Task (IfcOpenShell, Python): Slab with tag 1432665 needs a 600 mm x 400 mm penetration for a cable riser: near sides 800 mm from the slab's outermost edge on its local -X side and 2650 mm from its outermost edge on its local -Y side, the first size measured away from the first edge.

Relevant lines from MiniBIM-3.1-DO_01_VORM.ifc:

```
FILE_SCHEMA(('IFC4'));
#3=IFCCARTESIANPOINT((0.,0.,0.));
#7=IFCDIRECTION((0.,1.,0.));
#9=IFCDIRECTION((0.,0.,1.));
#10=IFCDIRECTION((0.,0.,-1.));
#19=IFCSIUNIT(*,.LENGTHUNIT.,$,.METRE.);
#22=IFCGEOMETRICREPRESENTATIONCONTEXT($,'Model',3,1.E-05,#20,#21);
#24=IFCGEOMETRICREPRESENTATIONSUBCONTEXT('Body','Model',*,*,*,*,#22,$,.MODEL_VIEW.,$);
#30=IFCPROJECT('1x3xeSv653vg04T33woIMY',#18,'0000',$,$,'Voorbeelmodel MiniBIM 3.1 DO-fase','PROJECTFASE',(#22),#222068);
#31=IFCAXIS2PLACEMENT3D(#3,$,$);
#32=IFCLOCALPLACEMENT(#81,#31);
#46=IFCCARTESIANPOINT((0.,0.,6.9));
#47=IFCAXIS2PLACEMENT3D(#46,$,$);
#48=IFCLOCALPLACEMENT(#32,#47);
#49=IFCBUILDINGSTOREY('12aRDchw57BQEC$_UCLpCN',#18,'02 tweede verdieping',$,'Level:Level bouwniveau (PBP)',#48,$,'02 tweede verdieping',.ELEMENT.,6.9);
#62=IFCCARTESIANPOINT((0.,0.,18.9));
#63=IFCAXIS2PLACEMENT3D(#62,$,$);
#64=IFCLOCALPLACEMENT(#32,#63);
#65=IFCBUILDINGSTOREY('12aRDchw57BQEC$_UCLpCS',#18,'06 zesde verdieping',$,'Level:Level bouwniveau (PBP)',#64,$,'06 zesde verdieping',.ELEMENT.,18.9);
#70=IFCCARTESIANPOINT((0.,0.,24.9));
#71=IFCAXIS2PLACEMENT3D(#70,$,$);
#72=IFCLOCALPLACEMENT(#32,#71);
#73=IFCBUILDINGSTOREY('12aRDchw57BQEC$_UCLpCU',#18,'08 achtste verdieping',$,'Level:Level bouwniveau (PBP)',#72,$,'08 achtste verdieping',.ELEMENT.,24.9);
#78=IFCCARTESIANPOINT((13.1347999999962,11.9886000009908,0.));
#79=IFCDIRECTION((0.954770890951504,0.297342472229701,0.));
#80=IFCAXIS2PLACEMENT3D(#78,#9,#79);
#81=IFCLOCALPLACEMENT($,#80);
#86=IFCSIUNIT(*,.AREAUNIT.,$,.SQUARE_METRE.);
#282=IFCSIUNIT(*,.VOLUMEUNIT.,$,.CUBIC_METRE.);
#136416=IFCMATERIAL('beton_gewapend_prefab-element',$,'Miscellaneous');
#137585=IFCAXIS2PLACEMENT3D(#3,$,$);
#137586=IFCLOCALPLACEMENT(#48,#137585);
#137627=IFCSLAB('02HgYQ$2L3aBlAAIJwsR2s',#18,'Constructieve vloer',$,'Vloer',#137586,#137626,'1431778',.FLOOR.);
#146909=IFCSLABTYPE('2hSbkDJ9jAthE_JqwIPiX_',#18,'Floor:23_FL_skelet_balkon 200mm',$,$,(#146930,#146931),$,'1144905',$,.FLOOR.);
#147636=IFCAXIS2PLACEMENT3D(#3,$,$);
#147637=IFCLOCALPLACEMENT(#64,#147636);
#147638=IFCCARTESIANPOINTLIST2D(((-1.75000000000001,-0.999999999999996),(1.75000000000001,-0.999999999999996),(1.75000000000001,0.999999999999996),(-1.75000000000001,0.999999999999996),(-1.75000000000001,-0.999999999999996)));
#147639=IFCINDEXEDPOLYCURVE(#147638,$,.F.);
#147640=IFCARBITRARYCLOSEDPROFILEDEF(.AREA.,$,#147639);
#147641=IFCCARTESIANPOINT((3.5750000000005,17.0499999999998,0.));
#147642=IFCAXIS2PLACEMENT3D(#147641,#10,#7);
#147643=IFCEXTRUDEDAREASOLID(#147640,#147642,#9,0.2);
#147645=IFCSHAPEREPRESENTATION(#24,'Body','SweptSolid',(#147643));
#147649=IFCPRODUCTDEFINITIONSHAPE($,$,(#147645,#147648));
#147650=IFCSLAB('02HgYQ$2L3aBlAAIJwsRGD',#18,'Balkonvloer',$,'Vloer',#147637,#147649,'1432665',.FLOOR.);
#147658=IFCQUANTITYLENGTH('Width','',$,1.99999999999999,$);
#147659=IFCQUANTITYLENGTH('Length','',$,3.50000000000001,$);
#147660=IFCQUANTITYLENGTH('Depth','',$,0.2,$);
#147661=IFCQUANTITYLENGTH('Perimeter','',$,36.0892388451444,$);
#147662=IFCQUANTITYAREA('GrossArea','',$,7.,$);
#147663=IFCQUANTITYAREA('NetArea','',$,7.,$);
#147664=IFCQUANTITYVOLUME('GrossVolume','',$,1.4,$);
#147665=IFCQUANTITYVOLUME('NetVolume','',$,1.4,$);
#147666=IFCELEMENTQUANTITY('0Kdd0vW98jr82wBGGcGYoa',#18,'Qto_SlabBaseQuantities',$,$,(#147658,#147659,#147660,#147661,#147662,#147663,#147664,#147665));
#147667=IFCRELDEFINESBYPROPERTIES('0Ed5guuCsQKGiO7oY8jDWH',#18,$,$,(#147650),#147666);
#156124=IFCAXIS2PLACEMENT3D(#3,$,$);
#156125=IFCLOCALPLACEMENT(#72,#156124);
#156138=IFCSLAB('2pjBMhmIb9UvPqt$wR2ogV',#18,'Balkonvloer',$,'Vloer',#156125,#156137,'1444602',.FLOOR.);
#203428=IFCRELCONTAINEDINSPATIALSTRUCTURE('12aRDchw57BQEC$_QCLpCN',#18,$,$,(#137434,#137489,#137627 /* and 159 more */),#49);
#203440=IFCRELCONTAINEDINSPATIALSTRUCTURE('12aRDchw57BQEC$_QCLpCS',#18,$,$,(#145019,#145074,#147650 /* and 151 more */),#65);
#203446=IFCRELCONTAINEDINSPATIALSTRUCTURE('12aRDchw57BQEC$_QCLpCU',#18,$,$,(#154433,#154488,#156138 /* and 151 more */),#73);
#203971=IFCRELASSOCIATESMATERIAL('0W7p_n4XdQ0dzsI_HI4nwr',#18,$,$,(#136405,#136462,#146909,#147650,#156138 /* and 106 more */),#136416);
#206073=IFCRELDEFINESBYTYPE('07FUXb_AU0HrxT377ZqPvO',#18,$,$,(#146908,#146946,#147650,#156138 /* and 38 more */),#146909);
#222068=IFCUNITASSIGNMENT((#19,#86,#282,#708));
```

```python
import numpy as np
import ifcopenshell
import ifcopenshell.api.feature
import ifcopenshell.api.geometry
import ifcopenshell.api.pset
import ifcopenshell.api.root
import ifcopenshell.geom
import ifcopenshell.util.element
import ifcopenshell.util.placement
import ifcopenshell.util.representation
import ifcopenshell.util.shape
import ifcopenshell.util.unit

model = ifcopenshell.open("MiniBIM-3.1-DO_01_VORM.ifc")
unit_scale = ifcopenshell.util.unit.calculate_unit_scale(model)
area_scale = ifcopenshell.util.unit.calculate_unit_scale(model, "AREAUNIT")
volume_scale = ifcopenshell.util.unit.calculate_unit_scale(model, "VOLUMEUNIT")
settings = ifcopenshell.geom.settings()


def volume(element):
    """Net volume in cubic metres, openings subtracted."""
    shape = ifcopenshell.geom.create_shape(settings, element)
    return ifcopenshell.util.shape.get_volume(shape.geometry)


slab = model.by_guid("02HgYQ$2L3aBlAAIJwsRGD")
before = volume(slab)

# Extent in the slab's own axes, in metres. The edges named are its -X and -Y sides.
slab_shape = ifcopenshell.geom.create_shape(settings, slab)
vertices = ifcopenshell.util.shape.get_vertices(slab_shape.geometry)
x_min, y_min, bottom = vertices.min(axis=0)
top = vertices[:, 2].max()

opening = ifcopenshell.api.root.create_entity(model, ifc_class="IfcOpeningElement", name="Cable riser opening", predefined_type="OPENING")
context = ifcopenshell.util.representation.get_context(model, "Model", "Body", "MODEL_VIEW")
width, depth = 0.6, 0.4
outline = [(0.0, 0.0), (width, 0.0), (width, depth), (0.0, depth), (0.0, 0.0)]
# Overshoot both faces by 50 mm so the cut is clean.
shape = ifcopenshell.api.geometry.add_slab_representation(
    model, context=context, depth=top - bottom + 0.1, polyline=outline
)
ifcopenshell.api.geometry.assign_representation(model, product=opening, representation=shape)

matrix = ifcopenshell.util.placement.get_local_placement(slab.ObjectPlacement)
matrix[:, 3] = matrix @ np.append(np.array([x_min + 0.8, y_min + 2.65, bottom - 0.05]) / unit_scale, 1.0)
ifcopenshell.api.geometry.edit_object_placement(model, product=opening, matrix=matrix, is_si=False)
ifcopenshell.api.feature.add_feature(model, feature=opening, element=slab)

after = volume(slab)

# Update the slab's stored quantities.
qto = model.by_id(ifcopenshell.util.element.get_pset(slab, "Qto_SlabBaseQuantities", should_inherit=False)["id"])
ifcopenshell.api.pset.edit_qto(model, qto=qto, properties={
    "NetArea": after / (top - bottom) / area_scale,
    "NetVolume": after / volume_scale,
})

print(f"slab volume {before:.3f} -> {after:.3f} m3")

model.write("MiniBIM-3.1-DO_01_VORM_edited.ifc")
```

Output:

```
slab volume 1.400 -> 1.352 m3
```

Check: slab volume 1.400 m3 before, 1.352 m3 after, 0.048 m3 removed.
